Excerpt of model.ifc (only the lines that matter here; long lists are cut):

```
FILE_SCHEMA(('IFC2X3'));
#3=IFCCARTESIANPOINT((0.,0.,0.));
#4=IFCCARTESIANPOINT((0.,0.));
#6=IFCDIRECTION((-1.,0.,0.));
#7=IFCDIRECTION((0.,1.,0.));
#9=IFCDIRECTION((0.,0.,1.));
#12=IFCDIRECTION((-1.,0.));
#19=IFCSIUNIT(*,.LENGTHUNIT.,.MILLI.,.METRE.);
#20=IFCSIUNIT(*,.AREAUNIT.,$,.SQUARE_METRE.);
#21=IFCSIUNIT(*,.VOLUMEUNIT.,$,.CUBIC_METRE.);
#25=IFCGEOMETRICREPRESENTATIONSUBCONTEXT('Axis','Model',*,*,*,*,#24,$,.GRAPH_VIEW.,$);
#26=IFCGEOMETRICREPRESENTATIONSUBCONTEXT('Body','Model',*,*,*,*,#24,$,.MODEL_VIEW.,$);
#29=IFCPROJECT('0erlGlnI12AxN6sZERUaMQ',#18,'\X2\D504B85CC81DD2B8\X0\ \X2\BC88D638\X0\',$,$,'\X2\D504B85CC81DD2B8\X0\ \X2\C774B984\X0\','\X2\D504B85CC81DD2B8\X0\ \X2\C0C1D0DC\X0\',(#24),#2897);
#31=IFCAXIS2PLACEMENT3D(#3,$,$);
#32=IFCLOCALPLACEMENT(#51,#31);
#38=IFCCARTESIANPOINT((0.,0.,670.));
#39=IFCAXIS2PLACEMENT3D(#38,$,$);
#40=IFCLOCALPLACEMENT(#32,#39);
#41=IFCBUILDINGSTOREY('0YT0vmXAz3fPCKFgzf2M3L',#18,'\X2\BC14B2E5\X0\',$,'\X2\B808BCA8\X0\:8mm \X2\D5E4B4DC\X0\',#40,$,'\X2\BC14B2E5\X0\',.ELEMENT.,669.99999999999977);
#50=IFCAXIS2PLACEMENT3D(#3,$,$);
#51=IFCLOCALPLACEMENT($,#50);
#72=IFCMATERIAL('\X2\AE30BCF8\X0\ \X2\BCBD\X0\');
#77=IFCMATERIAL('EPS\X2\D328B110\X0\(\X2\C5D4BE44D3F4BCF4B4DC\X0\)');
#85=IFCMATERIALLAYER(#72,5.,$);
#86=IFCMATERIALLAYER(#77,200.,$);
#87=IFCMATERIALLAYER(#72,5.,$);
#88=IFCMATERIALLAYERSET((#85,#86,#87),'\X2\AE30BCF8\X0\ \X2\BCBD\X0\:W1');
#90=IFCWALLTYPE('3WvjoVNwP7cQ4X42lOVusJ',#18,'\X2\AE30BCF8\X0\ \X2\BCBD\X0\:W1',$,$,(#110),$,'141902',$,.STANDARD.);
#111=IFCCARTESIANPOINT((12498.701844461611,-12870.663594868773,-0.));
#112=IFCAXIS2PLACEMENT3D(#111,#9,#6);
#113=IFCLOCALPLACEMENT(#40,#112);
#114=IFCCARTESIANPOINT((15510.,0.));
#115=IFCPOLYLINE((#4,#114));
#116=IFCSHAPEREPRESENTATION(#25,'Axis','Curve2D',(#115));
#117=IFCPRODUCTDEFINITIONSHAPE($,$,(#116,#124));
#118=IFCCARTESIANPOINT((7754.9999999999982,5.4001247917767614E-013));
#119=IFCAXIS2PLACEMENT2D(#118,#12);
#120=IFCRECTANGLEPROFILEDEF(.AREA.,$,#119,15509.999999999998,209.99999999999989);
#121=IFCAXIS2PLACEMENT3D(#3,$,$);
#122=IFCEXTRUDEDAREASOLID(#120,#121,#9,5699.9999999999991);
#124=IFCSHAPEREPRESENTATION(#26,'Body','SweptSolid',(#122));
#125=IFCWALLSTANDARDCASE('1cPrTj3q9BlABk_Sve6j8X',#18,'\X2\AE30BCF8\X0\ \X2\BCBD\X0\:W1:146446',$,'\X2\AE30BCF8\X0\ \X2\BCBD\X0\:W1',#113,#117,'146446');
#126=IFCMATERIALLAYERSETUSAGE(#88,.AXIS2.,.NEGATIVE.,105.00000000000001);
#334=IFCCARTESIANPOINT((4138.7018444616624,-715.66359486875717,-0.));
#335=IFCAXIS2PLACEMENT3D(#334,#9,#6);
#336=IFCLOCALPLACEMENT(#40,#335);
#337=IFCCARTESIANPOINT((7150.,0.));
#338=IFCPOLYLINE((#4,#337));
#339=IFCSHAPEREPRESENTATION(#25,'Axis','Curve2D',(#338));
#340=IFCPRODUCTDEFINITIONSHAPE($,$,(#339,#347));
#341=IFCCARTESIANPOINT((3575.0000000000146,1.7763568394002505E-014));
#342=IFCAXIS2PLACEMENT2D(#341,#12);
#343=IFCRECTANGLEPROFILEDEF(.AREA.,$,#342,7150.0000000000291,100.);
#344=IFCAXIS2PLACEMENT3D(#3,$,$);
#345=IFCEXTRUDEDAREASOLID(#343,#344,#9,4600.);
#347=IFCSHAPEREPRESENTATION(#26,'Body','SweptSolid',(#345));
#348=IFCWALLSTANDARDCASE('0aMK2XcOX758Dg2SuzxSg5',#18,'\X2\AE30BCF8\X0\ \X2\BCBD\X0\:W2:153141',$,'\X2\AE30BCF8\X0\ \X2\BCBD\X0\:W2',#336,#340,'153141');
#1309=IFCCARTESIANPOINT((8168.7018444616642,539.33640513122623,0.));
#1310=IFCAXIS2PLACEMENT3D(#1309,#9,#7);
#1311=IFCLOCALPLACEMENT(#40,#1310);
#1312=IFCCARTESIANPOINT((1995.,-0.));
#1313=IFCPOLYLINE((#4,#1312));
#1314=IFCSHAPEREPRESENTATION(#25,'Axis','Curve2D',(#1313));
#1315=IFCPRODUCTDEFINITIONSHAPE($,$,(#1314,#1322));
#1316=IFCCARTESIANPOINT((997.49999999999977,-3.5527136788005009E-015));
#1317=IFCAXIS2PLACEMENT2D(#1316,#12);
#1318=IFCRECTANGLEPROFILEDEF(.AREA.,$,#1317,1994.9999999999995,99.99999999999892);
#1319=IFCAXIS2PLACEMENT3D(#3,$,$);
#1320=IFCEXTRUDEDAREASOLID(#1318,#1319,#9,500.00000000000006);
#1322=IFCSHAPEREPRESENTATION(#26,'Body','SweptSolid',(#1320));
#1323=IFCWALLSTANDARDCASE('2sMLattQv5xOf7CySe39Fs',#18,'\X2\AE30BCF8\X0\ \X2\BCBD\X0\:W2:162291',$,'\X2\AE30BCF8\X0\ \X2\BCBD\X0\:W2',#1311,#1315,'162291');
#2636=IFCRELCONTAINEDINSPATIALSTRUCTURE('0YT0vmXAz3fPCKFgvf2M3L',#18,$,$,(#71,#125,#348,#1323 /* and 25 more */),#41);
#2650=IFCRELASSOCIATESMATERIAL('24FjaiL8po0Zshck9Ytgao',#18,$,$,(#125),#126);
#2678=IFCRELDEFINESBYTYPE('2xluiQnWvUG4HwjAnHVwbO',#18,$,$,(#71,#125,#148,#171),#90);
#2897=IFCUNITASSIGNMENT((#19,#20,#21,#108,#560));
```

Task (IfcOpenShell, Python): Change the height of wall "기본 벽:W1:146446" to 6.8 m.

```python
import ifcopenshell
import ifcopenshell.geom
import ifcopenshell.util.representation
import ifcopenshell.util.shape

model = ifcopenshell.open("model.ifc")
settings = ifcopenshell.geom.settings()


def volume(element):
    """Net volume in cubic metres, openings subtracted."""
    shape = ifcopenshell.geom.create_shape(settings, element)
    return ifcopenshell.util.shape.get_volume(shape.geometry)


wall = model.by_guid("1cPrTj3q9BlABk_Sve6j8X")
before = volume(wall)

body = ifcopenshell.util.representation.get_representation(wall, "Model", "Body")
solid = body.Items[0]
old_height = solid.Depth
solid.Depth = 6800.0
after = volume(wall)

print(f"height {old_height:g} -> {solid.Depth:g}, volume {before:.3f} -> {after:.3f} m3")

model.write("model_v2.ifc")
```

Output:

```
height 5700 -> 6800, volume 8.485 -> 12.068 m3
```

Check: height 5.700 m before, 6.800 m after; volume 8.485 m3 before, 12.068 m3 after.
